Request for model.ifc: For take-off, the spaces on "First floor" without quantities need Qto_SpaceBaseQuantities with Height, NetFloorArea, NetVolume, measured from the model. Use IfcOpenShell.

First a look at what the model holds.

```python
import ifcopenshell
import ifcopenshell.util.element
import ifcopenshell.util.unit

model = ifcopenshell.open("model.ifc")
print(model.schema)
for unit_type in ("LENGTHUNIT", "AREAUNIT", "VOLUMEUNIT"):
    print(unit_type, ifcopenshell.util.unit.calculate_unit_scale(model, unit_type))
storey = next(s for s in model.by_type("IfcBuildingStorey") if s.Name == "First floor")
spaces = [e for e in ifcopenshell.util.element.get_decomposition(storey) if e.is_a("IfcSpace")]
for e in sorted(spaces, key=lambda e: e.id()):
    print(e.id(), e.is_a(), e.Name, list(ifcopenshell.util.element.get_psets(e, qtos_only=True)), sep=" | ")
```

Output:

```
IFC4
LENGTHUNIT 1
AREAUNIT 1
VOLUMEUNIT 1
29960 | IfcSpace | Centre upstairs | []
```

```python
import ifcopenshell
import ifcopenshell.api.pset
import ifcopenshell.geom
import ifcopenshell.util.element
import ifcopenshell.util.shape
import ifcopenshell.util.unit

model = ifcopenshell.open("model.ifc")
unit_scale = ifcopenshell.util.unit.calculate_unit_scale(model)
area_scale = ifcopenshell.util.unit.calculate_unit_scale(model, "AREAUNIT")
volume_scale = ifcopenshell.util.unit.calculate_unit_scale(model, "VOLUMEUNIT")
settings = ifcopenshell.geom.settings()

storey = next(s for s in model.by_type("IfcBuildingStorey") if s.Name == "First floor")
spaces = [e for e in ifcopenshell.util.element.get_decomposition(storey) if e.is_a("IfcSpace")]

for e in sorted(spaces, key=lambda e: e.id()):
    if ifcopenshell.util.element.get_psets(e, qtos_only=True, should_inherit=False):
        continue
    # Geometry comes back in metres, in the element's own axes.
    shape = ifcopenshell.geom.create_shape(settings, e)
    values = {
        "Height": ifcopenshell.util.shape.get_z(shape.geometry) / unit_scale,
        "NetFloorArea": ifcopenshell.util.shape.get_footprint_area(shape.geometry) / area_scale,
        "NetVolume": ifcopenshell.util.shape.get_volume(shape.geometry) / volume_scale,
    }
    qto = ifcopenshell.api.pset.add_qto(model, product=e, name="Qto_SpaceBaseQuantities")
    ifcopenshell.api.pset.edit_qto(model, qto=qto, properties=values)
    print(e.id(), {k: round(v, 3) for k, v in values.items()})

model.write("model_v2.ifc")
```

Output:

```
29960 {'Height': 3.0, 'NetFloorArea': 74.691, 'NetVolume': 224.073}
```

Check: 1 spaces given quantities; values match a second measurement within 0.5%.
